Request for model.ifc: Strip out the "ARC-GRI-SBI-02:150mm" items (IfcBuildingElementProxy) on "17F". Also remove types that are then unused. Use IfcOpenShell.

First a look at what the model holds.

```python
import ifcopenshell
import ifcopenshell.util.element

model = ifcopenshell.open("model.ifc")
print(model.schema)
storey = next(s for s in model.by_type("IfcBuildingStorey") if s.Name == "17F")
proxies = [e for e in ifcopenshell.util.element.get_decomposition(storey) if e.is_a("IfcBuildingElementProxy")]
seen = {}
for e in proxies:
    element_type = ifcopenshell.util.element.get_type(e)
    name = element_type.Name if element_type not in (None, e) else None
    seen[name] = seen.get(name, 0) + 1
for name, count in sorted(seen.items(), key=str):
    print(count, "x", name)
```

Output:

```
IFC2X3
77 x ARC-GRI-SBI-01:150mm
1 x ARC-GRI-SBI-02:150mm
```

```python
import ifcopenshell
import ifcopenshell.api.root
import ifcopenshell.util.element

model = ifcopenshell.open("model.ifc")

storey = next(s for s in model.by_type("IfcBuildingStorey") if s.Name == "17F")
proxies = [e for e in ifcopenshell.util.element.get_decomposition(storey) if e.is_a("IfcBuildingElementProxy")]
targets = [e for e in proxies if (t := ifcopenshell.util.element.get_type(e)) not in (None, e) and t.Name == "ARC-GRI-SBI-02:150mm"]
types = {ifcopenshell.util.element.get_type(e) for e in targets} - {None, *targets}

for e in targets:
    ifcopenshell.api.root.remove_product(model, product=e)
print(len(targets), "removed")

unused = [t for t in types if not ifcopenshell.util.element.get_types(t)]
for t in unused:
    ifcopenshell.api.root.remove_product(model, product=t)
print(len(unused), "unused types removed")

model.write("model_edited.ifc")
```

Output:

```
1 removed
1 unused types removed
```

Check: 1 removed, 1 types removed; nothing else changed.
